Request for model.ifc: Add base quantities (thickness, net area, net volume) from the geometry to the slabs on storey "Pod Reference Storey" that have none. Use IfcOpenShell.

First a look at what the model holds.

```python
import ifcopenshell
import ifcopenshell.util.element
import ifcopenshell.util.unit

model = ifcopenshell.open("model.ifc")
print(model.schema)
for unit_type in ("LENGTHUNIT", "AREAUNIT", "VOLUMEUNIT"):
    print(unit_type, ifcopenshell.util.unit.calculate_unit_scale(model, unit_type))
storey = next(s for s in model.by_type("IfcBuildingStorey") if s.Name == "Pod Reference Storey")
slabs = [e for e in ifcopenshell.util.element.get_decomposition(storey) if e.is_a("IfcSlab")]
for e in sorted(slabs, key=lambda e: e.id()):
    print(e.id(), e.is_a(), e.Name, list(ifcopenshell.util.element.get_psets(e, qtos_only=True)), sep=" | ")
```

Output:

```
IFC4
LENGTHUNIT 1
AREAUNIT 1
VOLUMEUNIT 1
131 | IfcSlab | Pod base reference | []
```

```python
import ifcopenshell
import ifcopenshell.api.pset
import ifcopenshell.geom
import ifcopenshell.util.element
import ifcopenshell.util.shape
import ifcopenshell.util.unit

model = ifcopenshell.open("model.ifc")
unit_scale = ifcopenshell.util.unit.calculate_unit_scale(model)
area_scale = ifcopenshell.util.unit.calculate_unit_scale(model, "AREAUNIT")
volume_scale = ifcopenshell.util.unit.calculate_unit_scale(model, "VOLUMEUNIT")
settings = ifcopenshell.geom.settings()

storey = next(s for s in model.by_type("IfcBuildingStorey") if s.Name == "Pod Reference Storey")
slabs = [e for e in ifcopenshell.util.element.get_decomposition(storey) if e.is_a("IfcSlab")]

for e in sorted(slabs, key=lambda e: e.id()):
    if ifcopenshell.util.element.get_psets(e, qtos_only=True, should_inherit=False):
        continue
    # Geometry comes back in metres, in the element's own axes.
    shape = ifcopenshell.geom.create_shape(settings, e)
    values = {
        "Width": ifcopenshell.util.shape.get_z(shape.geometry) / unit_scale,
        "NetArea": ifcopenshell.util.shape.get_footprint_area(shape.geometry) / area_scale,
        "NetVolume": ifcopenshell.util.shape.get_volume(shape.geometry) / volume_scale,
    }
    qto = ifcopenshell.api.pset.add_qto(model, product=e, name="Qto_SlabBaseQuantities")
    ifcopenshell.api.pset.edit_qto(model, qto=qto, properties=values)
    print(e.id(), {k: round(v, 3) for k, v in values.items()})

model.write("model_rev.ifc")
```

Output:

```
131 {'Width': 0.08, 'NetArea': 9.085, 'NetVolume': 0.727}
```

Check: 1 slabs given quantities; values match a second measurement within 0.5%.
